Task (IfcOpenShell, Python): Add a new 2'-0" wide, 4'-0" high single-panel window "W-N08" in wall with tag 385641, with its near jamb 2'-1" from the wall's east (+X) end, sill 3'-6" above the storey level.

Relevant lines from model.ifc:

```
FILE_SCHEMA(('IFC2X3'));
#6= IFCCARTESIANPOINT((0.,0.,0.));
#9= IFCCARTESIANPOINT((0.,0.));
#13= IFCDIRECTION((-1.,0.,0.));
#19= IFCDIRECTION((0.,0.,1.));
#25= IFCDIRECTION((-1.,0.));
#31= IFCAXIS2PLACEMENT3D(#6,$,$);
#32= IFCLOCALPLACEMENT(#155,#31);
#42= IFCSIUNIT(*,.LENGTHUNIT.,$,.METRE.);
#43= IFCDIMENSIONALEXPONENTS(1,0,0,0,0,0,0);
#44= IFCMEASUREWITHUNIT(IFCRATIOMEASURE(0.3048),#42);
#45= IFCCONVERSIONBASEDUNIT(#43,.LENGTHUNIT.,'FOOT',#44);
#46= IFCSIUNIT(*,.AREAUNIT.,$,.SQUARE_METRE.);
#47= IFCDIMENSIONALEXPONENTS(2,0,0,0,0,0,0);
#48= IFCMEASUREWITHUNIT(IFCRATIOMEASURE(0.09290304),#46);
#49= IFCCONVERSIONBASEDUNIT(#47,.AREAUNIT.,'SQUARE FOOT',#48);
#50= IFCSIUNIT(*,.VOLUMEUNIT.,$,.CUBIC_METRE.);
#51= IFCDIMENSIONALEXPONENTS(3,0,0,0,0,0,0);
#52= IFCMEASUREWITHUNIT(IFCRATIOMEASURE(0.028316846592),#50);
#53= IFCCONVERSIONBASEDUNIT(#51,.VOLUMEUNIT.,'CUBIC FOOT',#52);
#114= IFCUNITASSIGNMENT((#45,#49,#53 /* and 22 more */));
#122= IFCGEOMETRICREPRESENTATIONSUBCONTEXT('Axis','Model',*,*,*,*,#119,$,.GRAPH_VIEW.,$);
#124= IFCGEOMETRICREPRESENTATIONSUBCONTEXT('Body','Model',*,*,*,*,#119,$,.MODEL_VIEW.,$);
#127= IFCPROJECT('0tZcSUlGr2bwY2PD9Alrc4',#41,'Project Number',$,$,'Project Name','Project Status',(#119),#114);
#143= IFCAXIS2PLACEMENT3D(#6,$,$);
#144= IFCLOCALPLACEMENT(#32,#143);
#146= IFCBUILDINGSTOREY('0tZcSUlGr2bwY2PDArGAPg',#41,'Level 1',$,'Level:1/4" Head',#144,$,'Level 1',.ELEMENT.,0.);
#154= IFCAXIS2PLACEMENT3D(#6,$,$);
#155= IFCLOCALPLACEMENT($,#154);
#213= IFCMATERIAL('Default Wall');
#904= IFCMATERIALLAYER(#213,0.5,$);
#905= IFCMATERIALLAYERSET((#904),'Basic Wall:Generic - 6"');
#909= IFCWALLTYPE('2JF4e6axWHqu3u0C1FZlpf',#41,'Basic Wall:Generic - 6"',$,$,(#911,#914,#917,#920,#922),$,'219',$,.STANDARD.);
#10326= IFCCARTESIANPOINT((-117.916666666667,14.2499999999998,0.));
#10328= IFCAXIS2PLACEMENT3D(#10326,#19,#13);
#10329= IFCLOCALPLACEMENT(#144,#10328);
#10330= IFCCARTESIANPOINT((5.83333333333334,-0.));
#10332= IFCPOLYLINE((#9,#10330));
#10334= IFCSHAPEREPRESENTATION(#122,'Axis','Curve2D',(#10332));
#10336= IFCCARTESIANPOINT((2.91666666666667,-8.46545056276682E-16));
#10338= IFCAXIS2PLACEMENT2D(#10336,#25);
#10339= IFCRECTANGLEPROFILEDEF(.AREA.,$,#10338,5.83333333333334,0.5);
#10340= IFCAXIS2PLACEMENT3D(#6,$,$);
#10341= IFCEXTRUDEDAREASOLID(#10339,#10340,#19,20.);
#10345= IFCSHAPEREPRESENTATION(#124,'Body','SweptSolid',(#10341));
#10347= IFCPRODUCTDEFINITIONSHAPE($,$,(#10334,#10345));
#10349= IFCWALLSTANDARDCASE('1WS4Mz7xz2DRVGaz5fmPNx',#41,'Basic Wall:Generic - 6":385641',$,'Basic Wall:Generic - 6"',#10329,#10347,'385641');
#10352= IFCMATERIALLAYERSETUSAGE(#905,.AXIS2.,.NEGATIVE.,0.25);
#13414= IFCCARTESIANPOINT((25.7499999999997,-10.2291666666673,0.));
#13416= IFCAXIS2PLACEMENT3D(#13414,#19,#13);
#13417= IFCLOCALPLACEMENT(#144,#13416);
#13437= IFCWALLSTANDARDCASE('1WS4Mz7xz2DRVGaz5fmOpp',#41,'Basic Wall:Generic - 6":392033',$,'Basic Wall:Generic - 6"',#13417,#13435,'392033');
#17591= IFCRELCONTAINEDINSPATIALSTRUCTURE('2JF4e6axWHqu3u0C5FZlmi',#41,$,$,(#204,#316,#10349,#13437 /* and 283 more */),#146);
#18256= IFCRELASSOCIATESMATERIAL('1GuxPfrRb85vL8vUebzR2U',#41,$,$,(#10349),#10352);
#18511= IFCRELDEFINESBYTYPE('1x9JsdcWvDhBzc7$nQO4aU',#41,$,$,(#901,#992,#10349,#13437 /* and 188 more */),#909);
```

```python
import numpy as np
import ifcopenshell
import ifcopenshell.api.feature
import ifcopenshell.api.geometry
import ifcopenshell.api.root
import ifcopenshell.api.spatial
import ifcopenshell.api.type
import ifcopenshell.geom
import ifcopenshell.util.element
import ifcopenshell.util.placement
import ifcopenshell.util.representation
import ifcopenshell.util.shape
import ifcopenshell.util.unit

model = ifcopenshell.open("model.ifc")
unit_scale = ifcopenshell.util.unit.calculate_unit_scale(model)
settings = ifcopenshell.geom.settings()


def volume(element):
    """Net volume in cubic metres, openings subtracted."""
    shape = ifcopenshell.geom.create_shape(settings, element)
    return ifcopenshell.util.shape.get_volume(shape.geometry)


wall = model.by_id(10349)
storey = ifcopenshell.util.element.get_container(wall, ifc_class="IfcBuildingStorey")
context = ifcopenshell.util.representation.get_context(model, "Model", "Body", "MODEL_VIEW")
before = volume(wall)

width, height, from_end, sill = 0.6096, 1.2192, 0.635, 1.0668  # metres

# The wall runs along its own X axis, and the end named is its -X end.
wall_shape = ifcopenshell.geom.create_shape(settings, wall)
x, y, z = ifcopenshell.util.shape.get_vertices(wall_shape.geometry).T
start = x.min() + from_end
face, thickness = float(y.min()), float(y.max() - y.min())
wall_matrix = ifcopenshell.util.placement.get_local_placement(wall.ObjectPlacement)
level = ifcopenshell.util.placement.get_local_placement(storey.ObjectPlacement)[2, 3]


def in_wall(x, y):
    """Placement at x, y metres in the wall's axes, at sill height."""
    matrix = wall_matrix.copy()
    matrix[:, 3] = wall_matrix @ np.array([x / unit_scale, y / unit_scale, 0.0, 1.0])
    matrix[2, 3] = level + sill / unit_scale
    return matrix


# Opening: a box that overshoots both wall faces by 50 mm.
opening = ifcopenshell.api.root.create_entity(model, ifc_class="IfcOpeningElement")
box = ifcopenshell.api.geometry.add_wall_representation(
    model, context=context, length=width, height=height, thickness=thickness + 0.1
)
ifcopenshell.api.geometry.assign_representation(model, product=opening, representation=box)
ifcopenshell.api.geometry.edit_object_placement(model, product=opening, matrix=in_wall(start, face - 0.05), is_si=False)
ifcopenshell.api.feature.add_feature(model, feature=opening, element=wall)

window = ifcopenshell.api.root.create_entity(model, ifc_class="IfcWindow", name="W-N08")
window.OverallWidth, window.OverallHeight = width / unit_scale, height / unit_scale
body = ifcopenshell.api.geometry.add_window_representation(
    model,
    context=context,
    overall_width=window.OverallWidth,
    overall_height=window.OverallHeight,
    partition_type="SINGLE_PANEL",
)
ifcopenshell.api.geometry.assign_representation(model, product=window, representation=body)
ifcopenshell.api.spatial.assign_container(model, products=[window], relating_structure=storey)
fills = ifcopenshell.api.feature.add_filling(model, opening=opening, element=window)
fills.OwnerHistory = window.OwnerHistory  # required in IFC2X3

# IFC2X3 keeps the operation on the window style.
style = ifcopenshell.api.root.create_entity(model, ifc_class="IfcWindowStyle", name="W-N08")
style.OperationType, style.ConstructionType = "SINGLE_PANEL", "NOTDEFINED"
style.ParameterTakesPrecedence = style.Sizeable = False
ifcopenshell.api.type.assign_type(model, related_objects=[window], relating_type=style)

# Centre the window in the wall's thickness.
ifcopenshell.api.geometry.edit_object_placement(model, product=window, matrix=in_wall(start, face), is_si=False)
window_shape = ifcopenshell.geom.create_shape(settings, window)
depth = ifcopenshell.util.shape.get_vertices(window_shape.geometry)[:, 1]
offset = face + thickness / 2 - (depth.min() + depth.max()) / 2
ifcopenshell.api.geometry.edit_object_placement(model, product=window, matrix=in_wall(start, offset), is_si=False)

after = volume(wall)

print(f"wall volume {before:.3f} -> {after:.3f} m3")

model.write("model_updated.ifc")
```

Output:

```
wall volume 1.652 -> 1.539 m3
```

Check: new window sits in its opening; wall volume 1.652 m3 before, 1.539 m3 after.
